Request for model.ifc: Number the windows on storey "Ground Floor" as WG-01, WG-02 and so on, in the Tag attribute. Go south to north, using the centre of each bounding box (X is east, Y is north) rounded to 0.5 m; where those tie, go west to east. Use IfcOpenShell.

First a look at what the model holds.

```python
import ifcopenshell
import ifcopenshell.util.element
import ifcopenshell.util.placement

model = ifcopenshell.open("model.ifc")
print(model.schema)
storey = next(s for s in model.by_type("IfcBuildingStorey") if s.Name == "Ground Floor")
windows = [e for e in ifcopenshell.util.element.get_decomposition(storey) if e.is_a("IfcWindow")]
for e in sorted(windows, key=lambda e: e.id()):
    origin = ifcopenshell.util.placement.get_local_placement(e.ObjectPlacement)[:3, 3]
    print(e.id(), e.Tag, e.Name, origin.round(2) + 0.0, sep=" | ")
```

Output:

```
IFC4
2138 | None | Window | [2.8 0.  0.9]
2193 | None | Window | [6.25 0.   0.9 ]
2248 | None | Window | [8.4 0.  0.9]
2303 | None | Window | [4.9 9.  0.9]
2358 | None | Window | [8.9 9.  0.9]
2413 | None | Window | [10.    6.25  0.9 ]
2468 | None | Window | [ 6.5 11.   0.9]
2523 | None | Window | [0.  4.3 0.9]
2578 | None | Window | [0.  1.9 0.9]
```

```python
import ifcopenshell
import ifcopenshell.geom
import ifcopenshell.util.element
import ifcopenshell.util.shape

model = ifcopenshell.open("model.ifc")
settings = ifcopenshell.geom.settings()
settings.set("use-world-coords", True)


def centre(element):
    shape = ifcopenshell.geom.create_shape(settings, element)
    return ifcopenshell.util.shape.get_bbox_centroid(shape.geometry)


storey = next(s for s in model.by_type("IfcBuildingStorey") if s.Name == "Ground Floor")
windows = [e for e in ifcopenshell.util.element.get_decomposition(storey) if e.is_a("IfcWindow")]

# Insertion points can sit at a corner or the storey origin, so sort by the geometry (in metres).
centres = {e: centre(e) for e in windows}
windows.sort(key=lambda e: (round(centres[e][1] / 0.5), centres[e][0]))

for i, e in enumerate(windows, start=1):
    number = f"WG-{i:02d}"
    e.Tag = number
    print(e.id(), number)

model.write("model_v2.ifc")
```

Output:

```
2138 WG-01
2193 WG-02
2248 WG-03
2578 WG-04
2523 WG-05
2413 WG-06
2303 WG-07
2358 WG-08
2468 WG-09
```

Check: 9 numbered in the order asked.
